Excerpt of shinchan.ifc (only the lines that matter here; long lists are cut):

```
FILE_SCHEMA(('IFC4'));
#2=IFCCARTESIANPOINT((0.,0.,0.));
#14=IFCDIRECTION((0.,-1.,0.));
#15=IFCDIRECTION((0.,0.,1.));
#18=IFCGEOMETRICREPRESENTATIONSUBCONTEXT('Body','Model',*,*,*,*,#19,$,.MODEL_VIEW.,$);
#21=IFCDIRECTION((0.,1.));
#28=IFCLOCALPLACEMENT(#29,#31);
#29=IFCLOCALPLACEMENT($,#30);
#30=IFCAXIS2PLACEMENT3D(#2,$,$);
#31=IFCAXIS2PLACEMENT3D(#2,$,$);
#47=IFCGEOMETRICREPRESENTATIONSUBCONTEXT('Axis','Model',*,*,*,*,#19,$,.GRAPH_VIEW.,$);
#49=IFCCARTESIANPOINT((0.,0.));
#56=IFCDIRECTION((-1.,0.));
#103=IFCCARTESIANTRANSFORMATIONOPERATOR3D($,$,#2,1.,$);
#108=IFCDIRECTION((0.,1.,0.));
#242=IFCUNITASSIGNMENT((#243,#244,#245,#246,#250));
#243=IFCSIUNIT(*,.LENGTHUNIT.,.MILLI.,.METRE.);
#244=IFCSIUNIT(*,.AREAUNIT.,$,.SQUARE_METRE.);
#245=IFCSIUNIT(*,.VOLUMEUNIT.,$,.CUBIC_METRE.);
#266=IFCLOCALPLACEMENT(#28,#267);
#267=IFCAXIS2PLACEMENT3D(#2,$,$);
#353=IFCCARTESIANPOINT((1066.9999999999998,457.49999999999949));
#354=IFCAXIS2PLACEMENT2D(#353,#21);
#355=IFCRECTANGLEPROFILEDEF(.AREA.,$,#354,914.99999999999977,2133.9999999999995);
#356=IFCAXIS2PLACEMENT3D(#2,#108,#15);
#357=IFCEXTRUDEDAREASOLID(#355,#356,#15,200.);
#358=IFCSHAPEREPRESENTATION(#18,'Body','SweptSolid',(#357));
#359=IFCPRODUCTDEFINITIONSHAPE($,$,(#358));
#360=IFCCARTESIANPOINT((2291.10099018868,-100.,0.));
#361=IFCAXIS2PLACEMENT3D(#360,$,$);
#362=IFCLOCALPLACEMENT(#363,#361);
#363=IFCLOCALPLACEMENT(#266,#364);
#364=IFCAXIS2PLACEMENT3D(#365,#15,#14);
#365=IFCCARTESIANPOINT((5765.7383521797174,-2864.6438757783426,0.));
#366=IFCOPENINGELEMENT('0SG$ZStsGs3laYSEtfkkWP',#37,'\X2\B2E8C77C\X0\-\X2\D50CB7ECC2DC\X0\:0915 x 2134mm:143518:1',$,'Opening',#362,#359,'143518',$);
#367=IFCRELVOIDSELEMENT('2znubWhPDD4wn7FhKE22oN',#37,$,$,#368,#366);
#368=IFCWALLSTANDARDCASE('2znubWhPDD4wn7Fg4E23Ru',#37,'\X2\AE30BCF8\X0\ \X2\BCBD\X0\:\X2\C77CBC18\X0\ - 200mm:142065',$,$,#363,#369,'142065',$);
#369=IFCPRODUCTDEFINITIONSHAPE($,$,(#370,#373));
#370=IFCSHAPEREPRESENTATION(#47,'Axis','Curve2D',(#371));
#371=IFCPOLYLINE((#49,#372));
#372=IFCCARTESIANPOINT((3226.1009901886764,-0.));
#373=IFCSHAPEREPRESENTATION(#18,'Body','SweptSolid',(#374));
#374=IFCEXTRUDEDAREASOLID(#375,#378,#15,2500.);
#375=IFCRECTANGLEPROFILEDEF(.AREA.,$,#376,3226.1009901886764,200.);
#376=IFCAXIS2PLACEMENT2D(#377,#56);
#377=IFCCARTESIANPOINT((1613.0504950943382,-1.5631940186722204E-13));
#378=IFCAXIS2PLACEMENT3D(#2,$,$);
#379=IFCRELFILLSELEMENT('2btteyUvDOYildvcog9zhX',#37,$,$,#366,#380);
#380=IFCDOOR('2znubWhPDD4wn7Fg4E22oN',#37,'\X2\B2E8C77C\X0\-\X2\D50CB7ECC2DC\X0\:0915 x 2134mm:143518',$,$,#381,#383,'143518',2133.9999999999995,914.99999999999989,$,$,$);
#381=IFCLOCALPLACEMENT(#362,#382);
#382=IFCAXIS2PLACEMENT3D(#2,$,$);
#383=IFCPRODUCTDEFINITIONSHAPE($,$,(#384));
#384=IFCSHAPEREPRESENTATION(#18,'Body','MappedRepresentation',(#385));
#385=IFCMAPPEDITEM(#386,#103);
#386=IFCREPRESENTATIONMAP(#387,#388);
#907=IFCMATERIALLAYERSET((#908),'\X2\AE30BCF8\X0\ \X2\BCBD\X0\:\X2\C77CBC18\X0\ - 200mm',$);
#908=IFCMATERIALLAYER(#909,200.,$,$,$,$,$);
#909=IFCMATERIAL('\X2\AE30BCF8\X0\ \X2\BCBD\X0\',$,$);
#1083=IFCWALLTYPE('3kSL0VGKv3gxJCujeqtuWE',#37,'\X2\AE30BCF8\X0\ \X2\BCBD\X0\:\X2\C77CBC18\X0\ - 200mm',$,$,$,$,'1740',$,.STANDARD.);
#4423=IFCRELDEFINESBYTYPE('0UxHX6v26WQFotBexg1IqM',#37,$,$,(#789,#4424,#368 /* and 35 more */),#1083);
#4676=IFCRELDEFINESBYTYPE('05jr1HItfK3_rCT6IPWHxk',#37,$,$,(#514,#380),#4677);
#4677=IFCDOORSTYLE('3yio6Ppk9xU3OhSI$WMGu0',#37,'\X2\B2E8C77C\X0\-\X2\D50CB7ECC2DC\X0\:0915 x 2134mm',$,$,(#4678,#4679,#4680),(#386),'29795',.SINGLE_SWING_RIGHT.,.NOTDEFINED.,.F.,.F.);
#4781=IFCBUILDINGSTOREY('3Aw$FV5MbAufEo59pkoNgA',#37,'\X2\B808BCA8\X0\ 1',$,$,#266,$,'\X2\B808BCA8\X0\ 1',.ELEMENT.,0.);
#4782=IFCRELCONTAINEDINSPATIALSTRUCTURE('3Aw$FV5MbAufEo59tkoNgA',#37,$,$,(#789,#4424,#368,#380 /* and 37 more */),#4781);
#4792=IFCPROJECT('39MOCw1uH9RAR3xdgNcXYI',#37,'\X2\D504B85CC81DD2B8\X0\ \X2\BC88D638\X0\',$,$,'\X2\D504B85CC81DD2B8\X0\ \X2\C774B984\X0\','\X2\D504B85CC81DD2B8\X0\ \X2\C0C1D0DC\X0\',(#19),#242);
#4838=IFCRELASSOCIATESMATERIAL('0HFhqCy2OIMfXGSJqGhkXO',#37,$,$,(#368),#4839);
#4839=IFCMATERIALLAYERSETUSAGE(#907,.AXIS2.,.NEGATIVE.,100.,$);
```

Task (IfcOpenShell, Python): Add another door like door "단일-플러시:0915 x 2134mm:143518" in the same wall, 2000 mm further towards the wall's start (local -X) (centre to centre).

```python
import ifcopenshell
import ifcopenshell.api.feature
import ifcopenshell.api.geometry
import ifcopenshell.api.root
import ifcopenshell.geom
import ifcopenshell.util.element
import ifcopenshell.util.placement
import ifcopenshell.util.shape
import ifcopenshell.util.unit

model = ifcopenshell.open("shinchan.ifc")
unit_scale = ifcopenshell.util.unit.calculate_unit_scale(model)
settings = ifcopenshell.geom.settings()


def volume(element):
    """Net volume in cubic metres, openings subtracted."""
    shape = ifcopenshell.geom.create_shape(settings, element)
    return ifcopenshell.util.shape.get_volume(shape.geometry)


def reuse_history(source, copy):
    """copy_class also copies each property set's owner history, people and application; keep the originals."""
    for rel in copy.IsDefinedBy:
        if rel.is_a("IfcRelDefinesByProperties") and (history := rel.RelatingPropertyDefinition.OwnerHistory):
            rel.RelatingPropertyDefinition.OwnerHistory = source.OwnerHistory
            ifcopenshell.util.element.remove_deep2(model, history)


door = model.by_id(380)
opening = door.FillsVoids[0].RelatingOpeningElement
wall = opening.VoidsElements[0].RelatingBuildingElement
before = volume(wall)
shift = ifcopenshell.util.placement.get_local_placement(wall.ObjectPlacement)[:3, 0] * -2 / unit_scale

# copy_class copies the void relationship, type, container and properties, but no geometry.
new_opening = ifcopenshell.api.root.copy_class(model, product=opening)
new_opening.Representation = ifcopenshell.util.element.copy_deep(
    model, opening.Representation, exclude=["IfcGeometricRepresentationContext", "IfcRepresentationMap"]
)
new_opening.Name = "단일-플러시:0915 x 2134mm"
new_opening.Tag = None
new_door = ifcopenshell.api.root.copy_class(model, product=door)
new_door.Representation = ifcopenshell.util.element.copy_deep(
    model, door.Representation, exclude=["IfcGeometricRepresentationContext", "IfcRepresentationMap"]
)
new_door.Name = "단일-플러시:0915 x 2134mm"
new_door.Tag = None
reuse_history(door, new_door)
ifcopenshell.api.feature.add_filling(model, opening=new_opening, element=new_door)

for old, new in ((opening, new_opening), (door, new_door)):
    matrix = ifcopenshell.util.placement.get_local_placement(old.ObjectPlacement)
    matrix[:3, 3] += shift
    ifcopenshell.api.geometry.edit_object_placement(model, product=new, matrix=matrix, is_si=False)

after = volume(wall)

print(f"wall volume {before:.3f} -> {after:.3f} m3")

model.write("shinchan_edited.ifc")
```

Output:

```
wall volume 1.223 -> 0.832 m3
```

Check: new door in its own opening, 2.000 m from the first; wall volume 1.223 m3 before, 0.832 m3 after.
